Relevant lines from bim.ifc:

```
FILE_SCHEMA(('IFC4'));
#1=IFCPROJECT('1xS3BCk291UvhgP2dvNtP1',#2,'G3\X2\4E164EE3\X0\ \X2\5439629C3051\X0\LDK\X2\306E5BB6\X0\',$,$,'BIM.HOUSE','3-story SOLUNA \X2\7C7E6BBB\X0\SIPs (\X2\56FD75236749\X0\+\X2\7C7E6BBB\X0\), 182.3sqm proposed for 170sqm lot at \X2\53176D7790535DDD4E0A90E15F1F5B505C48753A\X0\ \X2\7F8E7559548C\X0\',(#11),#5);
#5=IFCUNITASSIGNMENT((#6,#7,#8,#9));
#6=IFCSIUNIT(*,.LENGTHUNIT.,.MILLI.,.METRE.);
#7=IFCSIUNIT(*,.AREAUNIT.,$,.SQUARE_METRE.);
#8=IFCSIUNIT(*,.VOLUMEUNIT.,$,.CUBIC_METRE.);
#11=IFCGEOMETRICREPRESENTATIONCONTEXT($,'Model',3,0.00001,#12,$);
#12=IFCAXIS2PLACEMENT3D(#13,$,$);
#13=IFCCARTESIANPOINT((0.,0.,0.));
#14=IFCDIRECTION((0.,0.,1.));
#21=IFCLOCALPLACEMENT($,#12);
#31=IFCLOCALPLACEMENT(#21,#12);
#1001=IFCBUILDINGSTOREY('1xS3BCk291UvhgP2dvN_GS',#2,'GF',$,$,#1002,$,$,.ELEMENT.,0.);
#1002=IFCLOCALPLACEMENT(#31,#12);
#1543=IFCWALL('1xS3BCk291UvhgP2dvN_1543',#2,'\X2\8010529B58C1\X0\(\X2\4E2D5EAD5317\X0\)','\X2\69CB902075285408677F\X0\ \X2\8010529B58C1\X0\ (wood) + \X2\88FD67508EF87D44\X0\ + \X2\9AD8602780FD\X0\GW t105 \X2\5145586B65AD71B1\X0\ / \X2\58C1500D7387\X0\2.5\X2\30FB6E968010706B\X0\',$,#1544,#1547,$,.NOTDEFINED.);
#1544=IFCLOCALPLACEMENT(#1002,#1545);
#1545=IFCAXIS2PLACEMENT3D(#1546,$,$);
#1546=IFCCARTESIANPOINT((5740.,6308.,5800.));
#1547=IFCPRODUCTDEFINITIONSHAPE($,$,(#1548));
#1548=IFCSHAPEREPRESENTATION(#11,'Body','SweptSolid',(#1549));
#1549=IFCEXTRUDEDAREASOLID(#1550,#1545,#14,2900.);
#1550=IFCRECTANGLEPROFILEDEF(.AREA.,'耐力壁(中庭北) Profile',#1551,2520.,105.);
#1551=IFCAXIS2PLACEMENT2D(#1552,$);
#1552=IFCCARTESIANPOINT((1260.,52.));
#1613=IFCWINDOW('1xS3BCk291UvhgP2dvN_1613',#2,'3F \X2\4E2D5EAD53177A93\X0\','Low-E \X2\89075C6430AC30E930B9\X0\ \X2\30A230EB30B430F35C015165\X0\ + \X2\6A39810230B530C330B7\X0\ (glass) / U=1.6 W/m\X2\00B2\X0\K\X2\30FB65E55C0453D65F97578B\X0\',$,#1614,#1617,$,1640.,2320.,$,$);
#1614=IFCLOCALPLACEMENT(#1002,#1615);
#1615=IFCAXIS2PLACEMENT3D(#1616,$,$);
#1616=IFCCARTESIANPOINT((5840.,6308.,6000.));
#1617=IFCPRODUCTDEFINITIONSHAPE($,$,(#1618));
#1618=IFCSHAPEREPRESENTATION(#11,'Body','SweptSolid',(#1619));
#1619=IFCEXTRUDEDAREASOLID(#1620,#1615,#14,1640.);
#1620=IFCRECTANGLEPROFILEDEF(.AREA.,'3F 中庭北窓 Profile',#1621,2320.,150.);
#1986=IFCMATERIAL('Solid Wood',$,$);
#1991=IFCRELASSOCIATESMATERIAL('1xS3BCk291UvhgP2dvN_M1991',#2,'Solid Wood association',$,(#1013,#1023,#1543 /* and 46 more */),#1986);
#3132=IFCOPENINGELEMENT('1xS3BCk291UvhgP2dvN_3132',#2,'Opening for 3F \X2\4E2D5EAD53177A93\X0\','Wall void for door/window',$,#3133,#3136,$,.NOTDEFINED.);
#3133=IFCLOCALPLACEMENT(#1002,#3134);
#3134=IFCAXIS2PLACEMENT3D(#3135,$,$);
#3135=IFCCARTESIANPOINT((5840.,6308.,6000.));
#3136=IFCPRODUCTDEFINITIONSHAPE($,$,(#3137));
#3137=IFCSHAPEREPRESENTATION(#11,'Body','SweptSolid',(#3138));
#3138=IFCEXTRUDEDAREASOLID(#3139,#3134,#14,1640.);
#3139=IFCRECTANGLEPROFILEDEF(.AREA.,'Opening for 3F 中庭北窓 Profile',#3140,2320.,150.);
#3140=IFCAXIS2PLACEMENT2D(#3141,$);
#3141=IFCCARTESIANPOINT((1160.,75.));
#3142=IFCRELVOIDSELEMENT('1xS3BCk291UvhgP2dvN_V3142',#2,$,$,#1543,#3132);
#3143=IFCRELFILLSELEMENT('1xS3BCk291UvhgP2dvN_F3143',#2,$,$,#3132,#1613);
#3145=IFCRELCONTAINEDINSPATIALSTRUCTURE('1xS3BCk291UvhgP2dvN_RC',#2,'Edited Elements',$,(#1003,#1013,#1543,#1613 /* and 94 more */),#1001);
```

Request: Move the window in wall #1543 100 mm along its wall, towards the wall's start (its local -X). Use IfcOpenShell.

```python
import ifcopenshell
import ifcopenshell.api.geometry
import ifcopenshell.util.placement
import ifcopenshell.util.unit

model = ifcopenshell.open("bim.ifc")
unit_scale = ifcopenshell.util.unit.calculate_unit_scale(model)

window = model.by_id(1613)
opening = window.FillsVoids[0].RelatingOpeningElement
wall = opening.VoidsElements[0].RelatingBuildingElement

wall_matrix = ifcopenshell.util.placement.get_local_placement(wall.ObjectPlacement)
shift = wall_matrix[:3, 0] * -0.1 / unit_scale
before = ifcopenshell.util.placement.get_local_placement(window.ObjectPlacement)[:3, 3].copy()

# The window is not placed relative to its opening, so move both.
for product in (opening, window):
    matrix = ifcopenshell.util.placement.get_local_placement(product.ObjectPlacement)
    matrix[:3, 3] += shift
    ifcopenshell.api.geometry.edit_object_placement(model, product=product, matrix=matrix, is_si=False)

after = ifcopenshell.util.placement.get_local_placement(window.ObjectPlacement)[:3, 3]
print("window moved by", (after - before).round(3) + 0.0)

model.write("bim_edited.ifc")
```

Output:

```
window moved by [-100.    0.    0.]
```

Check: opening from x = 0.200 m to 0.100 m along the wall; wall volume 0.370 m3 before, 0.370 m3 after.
